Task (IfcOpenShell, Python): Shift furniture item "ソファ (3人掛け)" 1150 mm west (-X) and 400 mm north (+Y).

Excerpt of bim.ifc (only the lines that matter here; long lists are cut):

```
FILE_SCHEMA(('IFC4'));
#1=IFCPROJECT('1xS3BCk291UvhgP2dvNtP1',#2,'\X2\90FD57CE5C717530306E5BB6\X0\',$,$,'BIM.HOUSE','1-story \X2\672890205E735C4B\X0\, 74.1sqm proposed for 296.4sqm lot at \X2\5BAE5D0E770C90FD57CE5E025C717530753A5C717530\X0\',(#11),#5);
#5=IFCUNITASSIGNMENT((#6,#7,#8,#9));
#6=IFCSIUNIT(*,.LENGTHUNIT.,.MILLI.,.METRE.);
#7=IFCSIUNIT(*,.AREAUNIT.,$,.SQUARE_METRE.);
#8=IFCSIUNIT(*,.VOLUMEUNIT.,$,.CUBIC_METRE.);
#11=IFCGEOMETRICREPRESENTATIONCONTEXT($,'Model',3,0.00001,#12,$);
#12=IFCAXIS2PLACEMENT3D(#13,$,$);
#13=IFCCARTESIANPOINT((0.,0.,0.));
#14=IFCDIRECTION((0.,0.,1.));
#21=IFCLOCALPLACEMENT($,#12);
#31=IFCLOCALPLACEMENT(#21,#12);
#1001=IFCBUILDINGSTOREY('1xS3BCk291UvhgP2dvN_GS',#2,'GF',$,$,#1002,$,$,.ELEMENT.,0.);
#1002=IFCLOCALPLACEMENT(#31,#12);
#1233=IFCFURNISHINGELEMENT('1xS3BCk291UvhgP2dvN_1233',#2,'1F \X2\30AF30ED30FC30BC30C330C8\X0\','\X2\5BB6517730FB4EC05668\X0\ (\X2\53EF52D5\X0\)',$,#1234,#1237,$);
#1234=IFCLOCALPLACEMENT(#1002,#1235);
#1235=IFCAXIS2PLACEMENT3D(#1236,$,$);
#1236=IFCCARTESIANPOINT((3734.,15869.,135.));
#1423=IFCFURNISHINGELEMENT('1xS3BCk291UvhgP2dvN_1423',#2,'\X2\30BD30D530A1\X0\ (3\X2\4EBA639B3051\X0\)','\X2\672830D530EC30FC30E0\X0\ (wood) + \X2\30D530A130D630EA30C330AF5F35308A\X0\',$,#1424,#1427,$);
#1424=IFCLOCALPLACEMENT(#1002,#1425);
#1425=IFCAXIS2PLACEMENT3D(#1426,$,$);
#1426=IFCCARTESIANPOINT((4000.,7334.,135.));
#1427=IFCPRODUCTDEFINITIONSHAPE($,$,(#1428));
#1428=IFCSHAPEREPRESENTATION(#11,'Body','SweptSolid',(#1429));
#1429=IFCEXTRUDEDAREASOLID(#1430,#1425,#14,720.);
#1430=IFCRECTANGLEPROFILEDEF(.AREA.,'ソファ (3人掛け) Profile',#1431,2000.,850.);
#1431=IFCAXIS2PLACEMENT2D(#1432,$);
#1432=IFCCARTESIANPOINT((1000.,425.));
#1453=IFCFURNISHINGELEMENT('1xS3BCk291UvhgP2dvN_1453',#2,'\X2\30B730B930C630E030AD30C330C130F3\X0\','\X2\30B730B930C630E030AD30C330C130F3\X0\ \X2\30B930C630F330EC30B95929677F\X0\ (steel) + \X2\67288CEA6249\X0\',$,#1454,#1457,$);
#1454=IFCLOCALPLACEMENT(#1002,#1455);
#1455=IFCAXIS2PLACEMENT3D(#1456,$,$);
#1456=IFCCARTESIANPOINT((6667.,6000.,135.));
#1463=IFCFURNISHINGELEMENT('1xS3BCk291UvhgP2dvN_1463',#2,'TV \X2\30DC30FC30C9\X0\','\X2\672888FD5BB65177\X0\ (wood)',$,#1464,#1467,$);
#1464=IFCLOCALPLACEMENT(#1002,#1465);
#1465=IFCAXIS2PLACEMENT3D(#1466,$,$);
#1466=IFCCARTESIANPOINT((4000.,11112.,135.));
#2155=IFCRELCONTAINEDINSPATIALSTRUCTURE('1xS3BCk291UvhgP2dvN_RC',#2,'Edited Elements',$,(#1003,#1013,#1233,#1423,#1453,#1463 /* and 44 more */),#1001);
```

```python
import ifcopenshell
import ifcopenshell.api.geometry
import ifcopenshell.util.placement

model = ifcopenshell.open("bim.ifc")

item = model.by_guid("1xS3BCk291UvhgP2dvN_1423")
matrix = ifcopenshell.util.placement.get_local_placement(item.ObjectPlacement)
matrix[0, 3] -= 1150.0
matrix[1, 3] += 400.0
ifcopenshell.api.geometry.edit_object_placement(model, product=item, matrix=matrix, is_si=False)

print(ifcopenshell.util.placement.get_local_placement(item.ObjectPlacement).round(3) + 0.0)

model.write("bim_edited.ifc")
```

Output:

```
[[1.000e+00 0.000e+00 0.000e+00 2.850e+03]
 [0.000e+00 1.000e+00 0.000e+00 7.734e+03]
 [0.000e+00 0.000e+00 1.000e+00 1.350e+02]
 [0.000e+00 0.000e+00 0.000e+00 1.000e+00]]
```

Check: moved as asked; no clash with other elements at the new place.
